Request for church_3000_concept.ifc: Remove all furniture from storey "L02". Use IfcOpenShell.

First a look at what the model holds.

```python
import ifcopenshell
import ifcopenshell.util.element

model = ifcopenshell.open("church_3000_concept.ifc")
print(model.schema)
storey = next(s for s in model.by_type("IfcBuildingStorey") if s.Name == "L02")
furniture = [e for e in ifcopenshell.util.element.get_decomposition(storey) if e.is_a("IfcFurnishingElement")]
seen = {}
for e in furniture:
    element_type = ifcopenshell.util.element.get_type(e)
    name = element_type.Name if element_type not in (None, e) else None
    seen[name] = seen.get(name, 0) + 1
for name, count in sorted(seen.items(), key=str):
    print(count, "x", name)
```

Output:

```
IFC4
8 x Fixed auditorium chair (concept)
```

```python
import ifcopenshell
import ifcopenshell.api.root
import ifcopenshell.util.element

model = ifcopenshell.open("church_3000_concept.ifc")

storey = next(s for s in model.by_type("IfcBuildingStorey") if s.Name == "L02")
furniture = [e for e in ifcopenshell.util.element.get_decomposition(storey) if e.is_a("IfcFurnishingElement")]

for e in furniture:
    ifcopenshell.api.root.remove_product(model, product=e)
print(len(furniture), "removed")

model.write("church_3000_concept-out.ifc")
```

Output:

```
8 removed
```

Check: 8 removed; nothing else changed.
